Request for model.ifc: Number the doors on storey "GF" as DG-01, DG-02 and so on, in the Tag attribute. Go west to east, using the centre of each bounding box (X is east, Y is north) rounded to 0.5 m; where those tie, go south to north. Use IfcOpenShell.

First a look at what the model holds.

```python
import ifcopenshell
import ifcopenshell.util.element
import ifcopenshell.util.placement

model = ifcopenshell.open("model.ifc")
print(model.schema)
storey = next(s for s in model.by_type("IfcBuildingStorey") if s.Name == "GF")
doors = [e for e in ifcopenshell.util.element.get_decomposition(storey) if e.is_a("IfcDoor")]
for e in sorted(doors, key=lambda e: e.id()):
    origin = ifcopenshell.util.placement.get_local_placement(e.ObjectPlacement)[:3, 3]
    print(e.id(), e.Tag, e.Name, origin.round(2) + 0.0, sep=" | ")
```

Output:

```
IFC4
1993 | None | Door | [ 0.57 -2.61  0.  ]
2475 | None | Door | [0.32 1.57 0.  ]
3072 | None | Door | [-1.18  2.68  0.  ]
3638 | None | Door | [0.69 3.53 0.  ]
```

```python
import ifcopenshell
import ifcopenshell.geom
import ifcopenshell.util.element
import ifcopenshell.util.shape

model = ifcopenshell.open("model.ifc")
settings = ifcopenshell.geom.settings()
settings.set("use-world-coords", True)


def centre(element):
    shape = ifcopenshell.geom.create_shape(settings, element)
    return ifcopenshell.util.shape.get_bbox_centroid(shape.geometry)


storey = next(s for s in model.by_type("IfcBuildingStorey") if s.Name == "GF")
doors = [e for e in ifcopenshell.util.element.get_decomposition(storey) if e.is_a("IfcDoor")]

# Insertion points can sit at a corner or the storey origin, so sort by the geometry (in metres).
centres = {e: centre(e) for e in doors}
doors.sort(key=lambda e: (round(centres[e][0] / 0.5), centres[e][1]))

for i, e in enumerate(doors, start=1):
    number = f"DG-{i:02d}"
    e.Tag = number
    print(e.id(), number)

model.write("model_edited.ifc")
```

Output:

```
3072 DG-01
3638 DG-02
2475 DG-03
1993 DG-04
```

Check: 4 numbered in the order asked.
